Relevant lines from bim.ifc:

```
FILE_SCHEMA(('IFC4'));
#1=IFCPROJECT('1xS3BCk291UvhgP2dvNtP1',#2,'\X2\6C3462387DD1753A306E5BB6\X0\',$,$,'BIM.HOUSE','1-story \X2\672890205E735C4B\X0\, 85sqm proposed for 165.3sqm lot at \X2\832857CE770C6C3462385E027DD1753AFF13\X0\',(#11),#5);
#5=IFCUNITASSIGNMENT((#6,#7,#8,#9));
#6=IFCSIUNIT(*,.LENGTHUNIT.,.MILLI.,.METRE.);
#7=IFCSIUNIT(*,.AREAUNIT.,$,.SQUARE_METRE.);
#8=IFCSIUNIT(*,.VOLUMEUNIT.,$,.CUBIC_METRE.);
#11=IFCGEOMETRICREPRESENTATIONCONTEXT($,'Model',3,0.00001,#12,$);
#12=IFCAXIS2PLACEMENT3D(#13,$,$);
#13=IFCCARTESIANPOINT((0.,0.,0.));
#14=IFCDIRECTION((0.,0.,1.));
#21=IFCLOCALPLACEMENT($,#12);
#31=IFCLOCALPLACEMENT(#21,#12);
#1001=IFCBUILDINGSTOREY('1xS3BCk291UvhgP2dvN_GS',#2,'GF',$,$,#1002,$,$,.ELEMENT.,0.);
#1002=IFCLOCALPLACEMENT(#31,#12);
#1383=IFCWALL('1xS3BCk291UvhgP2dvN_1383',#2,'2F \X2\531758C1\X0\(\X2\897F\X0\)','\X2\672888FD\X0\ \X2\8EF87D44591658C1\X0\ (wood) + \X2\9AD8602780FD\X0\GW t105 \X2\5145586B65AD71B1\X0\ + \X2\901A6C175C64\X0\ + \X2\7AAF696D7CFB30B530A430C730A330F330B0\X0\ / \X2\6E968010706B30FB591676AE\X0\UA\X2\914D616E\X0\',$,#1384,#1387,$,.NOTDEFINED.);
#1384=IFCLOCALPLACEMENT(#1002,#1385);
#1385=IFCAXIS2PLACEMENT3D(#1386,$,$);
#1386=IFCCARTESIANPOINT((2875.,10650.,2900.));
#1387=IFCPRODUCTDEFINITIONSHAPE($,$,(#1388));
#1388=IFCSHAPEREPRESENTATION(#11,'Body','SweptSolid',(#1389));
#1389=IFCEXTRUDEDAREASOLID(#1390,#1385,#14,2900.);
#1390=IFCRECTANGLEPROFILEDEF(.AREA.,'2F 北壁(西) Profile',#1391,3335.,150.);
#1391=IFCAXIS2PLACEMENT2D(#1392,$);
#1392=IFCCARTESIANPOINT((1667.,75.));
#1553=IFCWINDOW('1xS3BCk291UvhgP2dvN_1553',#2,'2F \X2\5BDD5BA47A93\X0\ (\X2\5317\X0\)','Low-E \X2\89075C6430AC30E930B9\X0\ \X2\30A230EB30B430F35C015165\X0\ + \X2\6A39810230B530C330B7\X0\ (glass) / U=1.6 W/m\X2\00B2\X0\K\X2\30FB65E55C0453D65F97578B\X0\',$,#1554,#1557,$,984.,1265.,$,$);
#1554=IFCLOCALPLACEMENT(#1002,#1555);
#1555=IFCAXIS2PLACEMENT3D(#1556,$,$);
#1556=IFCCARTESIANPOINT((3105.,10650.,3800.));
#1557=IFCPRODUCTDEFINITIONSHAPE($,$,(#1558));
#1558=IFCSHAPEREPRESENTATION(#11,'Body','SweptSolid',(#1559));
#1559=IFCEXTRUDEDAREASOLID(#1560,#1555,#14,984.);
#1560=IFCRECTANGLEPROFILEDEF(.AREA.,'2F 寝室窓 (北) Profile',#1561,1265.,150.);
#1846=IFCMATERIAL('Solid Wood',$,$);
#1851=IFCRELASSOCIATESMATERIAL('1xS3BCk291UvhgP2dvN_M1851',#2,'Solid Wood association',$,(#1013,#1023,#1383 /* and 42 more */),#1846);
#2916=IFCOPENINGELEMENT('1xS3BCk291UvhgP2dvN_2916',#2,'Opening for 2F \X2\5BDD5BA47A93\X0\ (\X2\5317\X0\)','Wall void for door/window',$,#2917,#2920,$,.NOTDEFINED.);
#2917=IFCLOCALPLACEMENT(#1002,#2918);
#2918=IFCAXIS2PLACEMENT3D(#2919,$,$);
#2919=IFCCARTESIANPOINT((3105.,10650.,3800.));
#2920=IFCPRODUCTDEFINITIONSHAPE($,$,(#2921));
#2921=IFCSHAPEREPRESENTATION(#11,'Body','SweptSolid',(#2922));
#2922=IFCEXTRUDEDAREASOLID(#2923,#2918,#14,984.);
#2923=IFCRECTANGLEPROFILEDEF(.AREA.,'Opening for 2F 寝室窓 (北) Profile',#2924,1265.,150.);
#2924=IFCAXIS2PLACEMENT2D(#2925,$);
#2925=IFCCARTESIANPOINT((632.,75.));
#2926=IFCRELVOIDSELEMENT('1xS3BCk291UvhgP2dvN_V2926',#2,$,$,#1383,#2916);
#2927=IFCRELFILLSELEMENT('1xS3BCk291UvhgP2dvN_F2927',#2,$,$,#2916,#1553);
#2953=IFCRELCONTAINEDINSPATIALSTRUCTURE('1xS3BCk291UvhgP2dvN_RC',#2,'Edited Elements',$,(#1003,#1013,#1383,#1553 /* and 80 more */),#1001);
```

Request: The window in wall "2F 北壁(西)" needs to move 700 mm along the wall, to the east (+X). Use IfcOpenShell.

```python
import ifcopenshell
import ifcopenshell.api.geometry
import ifcopenshell.util.placement
import ifcopenshell.util.unit

model = ifcopenshell.open("bim.ifc")
unit_scale = ifcopenshell.util.unit.calculate_unit_scale(model)

window = model.by_id(1553)
opening = window.FillsVoids[0].RelatingOpeningElement
wall = opening.VoidsElements[0].RelatingBuildingElement

wall_matrix = ifcopenshell.util.placement.get_local_placement(wall.ObjectPlacement)
shift = wall_matrix[:3, 0] * 0.7 / unit_scale
before = ifcopenshell.util.placement.get_local_placement(window.ObjectPlacement)[:3, 3].copy()

# The window is not placed relative to its opening, so move both.
for product in (opening, window):
    matrix = ifcopenshell.util.placement.get_local_placement(product.ObjectPlacement)
    matrix[:3, 3] += shift
    ifcopenshell.api.geometry.edit_object_placement(model, product=product, matrix=matrix, is_si=False)

after = ifcopenshell.util.placement.get_local_placement(window.ObjectPlacement)[:3, 3]
print("window moved by", (after - before).round(3) + 0.0)

model.write("bim-out.ifc")
```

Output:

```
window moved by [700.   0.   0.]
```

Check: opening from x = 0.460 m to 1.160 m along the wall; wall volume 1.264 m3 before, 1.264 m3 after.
